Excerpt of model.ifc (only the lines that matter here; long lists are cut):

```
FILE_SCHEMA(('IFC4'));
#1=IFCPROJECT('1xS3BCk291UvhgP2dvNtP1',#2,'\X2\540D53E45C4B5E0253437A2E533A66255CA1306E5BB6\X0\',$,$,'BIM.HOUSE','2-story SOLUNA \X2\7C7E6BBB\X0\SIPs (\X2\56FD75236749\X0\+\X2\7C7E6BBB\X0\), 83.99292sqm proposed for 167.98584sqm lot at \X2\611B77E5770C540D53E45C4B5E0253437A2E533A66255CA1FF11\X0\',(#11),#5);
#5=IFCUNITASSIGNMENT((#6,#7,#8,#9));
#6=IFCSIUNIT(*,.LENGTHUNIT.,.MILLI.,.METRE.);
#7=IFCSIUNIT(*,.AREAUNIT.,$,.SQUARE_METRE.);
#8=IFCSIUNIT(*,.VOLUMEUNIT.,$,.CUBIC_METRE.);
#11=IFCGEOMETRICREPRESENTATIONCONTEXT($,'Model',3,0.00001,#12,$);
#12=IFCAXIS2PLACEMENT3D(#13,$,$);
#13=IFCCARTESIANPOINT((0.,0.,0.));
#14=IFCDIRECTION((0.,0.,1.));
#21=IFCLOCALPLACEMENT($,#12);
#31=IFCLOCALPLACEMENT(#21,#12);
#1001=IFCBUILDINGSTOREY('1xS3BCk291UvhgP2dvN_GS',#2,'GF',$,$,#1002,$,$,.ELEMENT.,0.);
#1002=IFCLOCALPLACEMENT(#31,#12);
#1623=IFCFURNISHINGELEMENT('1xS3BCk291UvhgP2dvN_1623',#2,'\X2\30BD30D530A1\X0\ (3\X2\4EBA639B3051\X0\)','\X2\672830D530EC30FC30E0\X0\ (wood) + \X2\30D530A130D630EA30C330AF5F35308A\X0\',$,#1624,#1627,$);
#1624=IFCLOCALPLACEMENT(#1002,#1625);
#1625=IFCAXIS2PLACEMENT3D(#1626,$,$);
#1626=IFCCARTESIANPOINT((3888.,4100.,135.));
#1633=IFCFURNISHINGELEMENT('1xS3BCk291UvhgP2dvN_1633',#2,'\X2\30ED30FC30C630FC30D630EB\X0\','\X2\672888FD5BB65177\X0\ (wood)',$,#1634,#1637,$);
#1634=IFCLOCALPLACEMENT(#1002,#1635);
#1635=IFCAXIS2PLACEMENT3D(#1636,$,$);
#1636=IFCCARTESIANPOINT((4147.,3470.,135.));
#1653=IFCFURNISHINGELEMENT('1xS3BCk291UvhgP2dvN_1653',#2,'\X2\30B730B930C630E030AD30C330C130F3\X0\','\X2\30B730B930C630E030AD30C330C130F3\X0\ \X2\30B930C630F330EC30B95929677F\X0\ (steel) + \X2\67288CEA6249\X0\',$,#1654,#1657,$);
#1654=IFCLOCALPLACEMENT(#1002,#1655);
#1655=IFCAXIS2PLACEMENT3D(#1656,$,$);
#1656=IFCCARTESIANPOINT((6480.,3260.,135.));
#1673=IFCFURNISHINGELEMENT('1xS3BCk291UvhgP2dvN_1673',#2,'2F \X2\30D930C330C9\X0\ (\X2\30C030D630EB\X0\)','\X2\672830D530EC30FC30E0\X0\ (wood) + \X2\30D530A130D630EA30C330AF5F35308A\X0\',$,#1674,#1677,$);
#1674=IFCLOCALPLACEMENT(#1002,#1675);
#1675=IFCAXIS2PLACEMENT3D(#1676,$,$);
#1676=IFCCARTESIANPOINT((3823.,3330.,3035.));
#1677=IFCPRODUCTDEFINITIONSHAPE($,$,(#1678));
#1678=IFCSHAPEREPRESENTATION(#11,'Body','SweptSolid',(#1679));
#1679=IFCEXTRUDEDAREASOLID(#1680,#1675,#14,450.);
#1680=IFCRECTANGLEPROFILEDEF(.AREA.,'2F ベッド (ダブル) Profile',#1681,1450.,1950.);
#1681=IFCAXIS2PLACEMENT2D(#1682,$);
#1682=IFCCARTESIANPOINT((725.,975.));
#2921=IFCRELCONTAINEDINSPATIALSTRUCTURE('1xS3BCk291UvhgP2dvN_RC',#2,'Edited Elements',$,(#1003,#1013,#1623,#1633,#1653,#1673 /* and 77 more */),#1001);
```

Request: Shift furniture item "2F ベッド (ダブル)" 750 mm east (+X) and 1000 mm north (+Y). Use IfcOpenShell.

```python
import ifcopenshell
import ifcopenshell.api.geometry
import ifcopenshell.util.placement
import ifcopenshell.util.unit

model = ifcopenshell.open("model.ifc")
unit_scale = ifcopenshell.util.unit.calculate_unit_scale(model)

item = model.by_id(1673)
matrix = ifcopenshell.util.placement.get_local_placement(item.ObjectPlacement)
matrix[0, 3] += 0.75 / unit_scale
matrix[1, 3] += 1 / unit_scale
ifcopenshell.api.geometry.edit_object_placement(model, product=item, matrix=matrix, is_si=False)

print(ifcopenshell.util.placement.get_local_placement(item.ObjectPlacement).round(3) + 0.0)

model.write("model_v2.ifc")
```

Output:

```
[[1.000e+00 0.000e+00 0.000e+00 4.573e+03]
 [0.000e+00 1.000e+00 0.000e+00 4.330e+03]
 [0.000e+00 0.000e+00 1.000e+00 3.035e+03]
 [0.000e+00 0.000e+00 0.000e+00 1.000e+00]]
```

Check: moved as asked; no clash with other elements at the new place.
